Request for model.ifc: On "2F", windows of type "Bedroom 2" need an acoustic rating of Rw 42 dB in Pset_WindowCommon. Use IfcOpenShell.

First a look at what the model holds.

```python
import ifcopenshell
import ifcopenshell.util.element

model = ifcopenshell.open("model.ifc")
print(model.schema)
storey = next(s for s in model.by_type("IfcBuildingStorey") if s.Name == "2F")
windows = [e for e in ifcopenshell.util.element.get_decomposition(storey) if e.is_a("IfcWindow")]
seen = {}
for e in windows:
    element_type = ifcopenshell.util.element.get_type(e)
    key = (element_type.Name if element_type != e and element_type else None, ifcopenshell.util.element.get_pset(e, "Pset_WindowCommon", "AcousticRating"))
    seen[key] = seen.get(key, 0) + 1
for (name, value), count in sorted(seen.items(), key=str):
    print(count, "x", name, "|", value)
```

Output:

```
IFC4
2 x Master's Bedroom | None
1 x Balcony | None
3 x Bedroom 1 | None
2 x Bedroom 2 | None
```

```python
import ifcopenshell
import ifcopenshell.api.pset
import ifcopenshell.util.element

model = ifcopenshell.open("model.ifc")

storey = next(s for s in model.by_type("IfcBuildingStorey") if s.Name == "2F")
windows = [e for e in ifcopenshell.util.element.get_decomposition(storey) if e.is_a("IfcWindow")]

count = 0
for e in windows:
    element_type = ifcopenshell.util.element.get_type(e)
    if element_type in (None, e) or element_type.Name != "Bedroom 2":
        continue
    # add_pset returns the element's existing set when there is one.
    pset = ifcopenshell.api.pset.add_pset(model, product=e, name="Pset_WindowCommon")
    ifcopenshell.api.pset.edit_pset(model, pset=pset, properties={"AcousticRating": "Rw 42 dB"})
    count += 1

print(count, "windows updated")

model.write("model_v2.ifc")
```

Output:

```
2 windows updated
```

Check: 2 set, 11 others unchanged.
